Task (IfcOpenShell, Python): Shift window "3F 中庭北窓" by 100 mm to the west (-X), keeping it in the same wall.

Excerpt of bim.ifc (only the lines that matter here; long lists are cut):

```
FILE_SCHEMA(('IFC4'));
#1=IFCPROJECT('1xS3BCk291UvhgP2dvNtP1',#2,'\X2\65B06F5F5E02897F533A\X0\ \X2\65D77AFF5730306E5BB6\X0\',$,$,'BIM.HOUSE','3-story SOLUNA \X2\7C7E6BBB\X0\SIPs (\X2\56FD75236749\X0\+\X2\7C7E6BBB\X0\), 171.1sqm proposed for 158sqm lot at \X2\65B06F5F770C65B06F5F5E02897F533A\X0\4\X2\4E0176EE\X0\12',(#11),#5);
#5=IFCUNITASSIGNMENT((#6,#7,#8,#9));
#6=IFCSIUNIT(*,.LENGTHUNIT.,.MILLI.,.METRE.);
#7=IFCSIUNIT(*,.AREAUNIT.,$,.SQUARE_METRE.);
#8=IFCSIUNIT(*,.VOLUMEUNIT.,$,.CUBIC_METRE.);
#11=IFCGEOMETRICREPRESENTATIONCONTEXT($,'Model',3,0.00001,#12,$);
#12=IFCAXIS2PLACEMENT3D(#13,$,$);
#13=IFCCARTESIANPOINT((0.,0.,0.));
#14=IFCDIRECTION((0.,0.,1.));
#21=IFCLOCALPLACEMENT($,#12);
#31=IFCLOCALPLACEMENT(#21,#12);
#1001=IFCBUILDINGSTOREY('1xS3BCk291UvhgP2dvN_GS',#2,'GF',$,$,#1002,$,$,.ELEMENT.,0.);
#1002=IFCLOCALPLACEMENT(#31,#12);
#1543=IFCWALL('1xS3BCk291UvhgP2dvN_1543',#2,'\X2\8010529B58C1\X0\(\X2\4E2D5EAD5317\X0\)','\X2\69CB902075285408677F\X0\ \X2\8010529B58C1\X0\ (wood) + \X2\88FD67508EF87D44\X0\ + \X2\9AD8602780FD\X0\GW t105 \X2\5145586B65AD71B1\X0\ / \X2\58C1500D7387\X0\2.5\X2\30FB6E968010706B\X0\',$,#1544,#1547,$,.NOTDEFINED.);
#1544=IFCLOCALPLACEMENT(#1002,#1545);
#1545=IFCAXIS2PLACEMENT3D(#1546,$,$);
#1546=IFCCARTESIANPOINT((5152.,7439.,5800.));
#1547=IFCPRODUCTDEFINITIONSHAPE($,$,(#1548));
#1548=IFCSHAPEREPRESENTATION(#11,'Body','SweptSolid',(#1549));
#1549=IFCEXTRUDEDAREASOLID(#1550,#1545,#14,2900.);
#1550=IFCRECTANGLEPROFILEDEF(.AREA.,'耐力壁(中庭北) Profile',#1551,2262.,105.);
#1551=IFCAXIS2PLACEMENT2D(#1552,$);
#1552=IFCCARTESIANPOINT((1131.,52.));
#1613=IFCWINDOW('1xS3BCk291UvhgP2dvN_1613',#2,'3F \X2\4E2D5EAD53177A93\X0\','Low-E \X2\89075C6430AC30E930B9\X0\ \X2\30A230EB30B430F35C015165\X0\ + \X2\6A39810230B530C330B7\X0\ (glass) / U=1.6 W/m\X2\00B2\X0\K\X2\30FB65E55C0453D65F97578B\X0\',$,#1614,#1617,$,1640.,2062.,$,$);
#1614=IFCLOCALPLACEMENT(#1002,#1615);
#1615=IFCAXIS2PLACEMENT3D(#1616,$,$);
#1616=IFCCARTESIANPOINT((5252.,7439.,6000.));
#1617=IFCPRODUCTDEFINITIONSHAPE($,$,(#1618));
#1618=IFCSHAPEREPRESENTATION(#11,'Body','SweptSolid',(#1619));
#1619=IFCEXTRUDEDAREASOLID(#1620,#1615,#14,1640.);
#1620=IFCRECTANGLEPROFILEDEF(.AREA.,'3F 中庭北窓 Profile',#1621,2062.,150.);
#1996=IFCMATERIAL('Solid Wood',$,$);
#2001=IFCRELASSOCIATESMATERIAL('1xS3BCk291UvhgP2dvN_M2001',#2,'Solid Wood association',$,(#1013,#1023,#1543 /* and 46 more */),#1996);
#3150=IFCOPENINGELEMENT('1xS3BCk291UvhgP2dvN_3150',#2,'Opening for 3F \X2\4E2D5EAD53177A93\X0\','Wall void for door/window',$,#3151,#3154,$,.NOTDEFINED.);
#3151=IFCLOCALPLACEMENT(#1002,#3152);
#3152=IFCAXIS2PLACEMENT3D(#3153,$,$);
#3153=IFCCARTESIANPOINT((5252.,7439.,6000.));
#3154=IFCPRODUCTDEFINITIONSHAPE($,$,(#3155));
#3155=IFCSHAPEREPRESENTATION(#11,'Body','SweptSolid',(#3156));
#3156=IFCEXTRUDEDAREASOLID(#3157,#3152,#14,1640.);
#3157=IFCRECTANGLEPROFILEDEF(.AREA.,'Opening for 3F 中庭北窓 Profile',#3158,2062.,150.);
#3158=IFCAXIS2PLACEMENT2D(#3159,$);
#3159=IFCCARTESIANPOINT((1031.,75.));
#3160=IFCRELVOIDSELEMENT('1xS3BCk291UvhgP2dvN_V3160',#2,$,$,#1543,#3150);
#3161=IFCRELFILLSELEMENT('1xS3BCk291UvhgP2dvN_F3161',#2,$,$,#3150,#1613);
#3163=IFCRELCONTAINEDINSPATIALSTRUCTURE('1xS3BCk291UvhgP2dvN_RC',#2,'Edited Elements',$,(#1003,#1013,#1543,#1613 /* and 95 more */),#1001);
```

```python
import ifcopenshell
import ifcopenshell.api.geometry
import ifcopenshell.util.placement
import ifcopenshell.util.unit

model = ifcopenshell.open("bim.ifc")
unit_scale = ifcopenshell.util.unit.calculate_unit_scale(model)

window = model.by_guid("1xS3BCk291UvhgP2dvN_1613")
opening = window.FillsVoids[0].RelatingOpeningElement
wall = opening.VoidsElements[0].RelatingBuildingElement

wall_matrix = ifcopenshell.util.placement.get_local_placement(wall.ObjectPlacement)
shift = wall_matrix[:3, 0] * -0.1 / unit_scale
before = ifcopenshell.util.placement.get_local_placement(window.ObjectPlacement)[:3, 3].copy()

# The window is not placed relative to its opening, so move both.
for product in (opening, window):
    matrix = ifcopenshell.util.placement.get_local_placement(product.ObjectPlacement)
    matrix[:3, 3] += shift
    ifcopenshell.api.geometry.edit_object_placement(model, product=product, matrix=matrix, is_si=False)

after = ifcopenshell.util.placement.get_local_placement(window.ObjectPlacement)[:3, 3]
print("window moved by", (after - before).round(3) + 0.0)

model.write("bim-out.ifc")
```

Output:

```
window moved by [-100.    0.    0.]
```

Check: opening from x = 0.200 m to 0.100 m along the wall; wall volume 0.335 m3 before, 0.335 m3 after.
